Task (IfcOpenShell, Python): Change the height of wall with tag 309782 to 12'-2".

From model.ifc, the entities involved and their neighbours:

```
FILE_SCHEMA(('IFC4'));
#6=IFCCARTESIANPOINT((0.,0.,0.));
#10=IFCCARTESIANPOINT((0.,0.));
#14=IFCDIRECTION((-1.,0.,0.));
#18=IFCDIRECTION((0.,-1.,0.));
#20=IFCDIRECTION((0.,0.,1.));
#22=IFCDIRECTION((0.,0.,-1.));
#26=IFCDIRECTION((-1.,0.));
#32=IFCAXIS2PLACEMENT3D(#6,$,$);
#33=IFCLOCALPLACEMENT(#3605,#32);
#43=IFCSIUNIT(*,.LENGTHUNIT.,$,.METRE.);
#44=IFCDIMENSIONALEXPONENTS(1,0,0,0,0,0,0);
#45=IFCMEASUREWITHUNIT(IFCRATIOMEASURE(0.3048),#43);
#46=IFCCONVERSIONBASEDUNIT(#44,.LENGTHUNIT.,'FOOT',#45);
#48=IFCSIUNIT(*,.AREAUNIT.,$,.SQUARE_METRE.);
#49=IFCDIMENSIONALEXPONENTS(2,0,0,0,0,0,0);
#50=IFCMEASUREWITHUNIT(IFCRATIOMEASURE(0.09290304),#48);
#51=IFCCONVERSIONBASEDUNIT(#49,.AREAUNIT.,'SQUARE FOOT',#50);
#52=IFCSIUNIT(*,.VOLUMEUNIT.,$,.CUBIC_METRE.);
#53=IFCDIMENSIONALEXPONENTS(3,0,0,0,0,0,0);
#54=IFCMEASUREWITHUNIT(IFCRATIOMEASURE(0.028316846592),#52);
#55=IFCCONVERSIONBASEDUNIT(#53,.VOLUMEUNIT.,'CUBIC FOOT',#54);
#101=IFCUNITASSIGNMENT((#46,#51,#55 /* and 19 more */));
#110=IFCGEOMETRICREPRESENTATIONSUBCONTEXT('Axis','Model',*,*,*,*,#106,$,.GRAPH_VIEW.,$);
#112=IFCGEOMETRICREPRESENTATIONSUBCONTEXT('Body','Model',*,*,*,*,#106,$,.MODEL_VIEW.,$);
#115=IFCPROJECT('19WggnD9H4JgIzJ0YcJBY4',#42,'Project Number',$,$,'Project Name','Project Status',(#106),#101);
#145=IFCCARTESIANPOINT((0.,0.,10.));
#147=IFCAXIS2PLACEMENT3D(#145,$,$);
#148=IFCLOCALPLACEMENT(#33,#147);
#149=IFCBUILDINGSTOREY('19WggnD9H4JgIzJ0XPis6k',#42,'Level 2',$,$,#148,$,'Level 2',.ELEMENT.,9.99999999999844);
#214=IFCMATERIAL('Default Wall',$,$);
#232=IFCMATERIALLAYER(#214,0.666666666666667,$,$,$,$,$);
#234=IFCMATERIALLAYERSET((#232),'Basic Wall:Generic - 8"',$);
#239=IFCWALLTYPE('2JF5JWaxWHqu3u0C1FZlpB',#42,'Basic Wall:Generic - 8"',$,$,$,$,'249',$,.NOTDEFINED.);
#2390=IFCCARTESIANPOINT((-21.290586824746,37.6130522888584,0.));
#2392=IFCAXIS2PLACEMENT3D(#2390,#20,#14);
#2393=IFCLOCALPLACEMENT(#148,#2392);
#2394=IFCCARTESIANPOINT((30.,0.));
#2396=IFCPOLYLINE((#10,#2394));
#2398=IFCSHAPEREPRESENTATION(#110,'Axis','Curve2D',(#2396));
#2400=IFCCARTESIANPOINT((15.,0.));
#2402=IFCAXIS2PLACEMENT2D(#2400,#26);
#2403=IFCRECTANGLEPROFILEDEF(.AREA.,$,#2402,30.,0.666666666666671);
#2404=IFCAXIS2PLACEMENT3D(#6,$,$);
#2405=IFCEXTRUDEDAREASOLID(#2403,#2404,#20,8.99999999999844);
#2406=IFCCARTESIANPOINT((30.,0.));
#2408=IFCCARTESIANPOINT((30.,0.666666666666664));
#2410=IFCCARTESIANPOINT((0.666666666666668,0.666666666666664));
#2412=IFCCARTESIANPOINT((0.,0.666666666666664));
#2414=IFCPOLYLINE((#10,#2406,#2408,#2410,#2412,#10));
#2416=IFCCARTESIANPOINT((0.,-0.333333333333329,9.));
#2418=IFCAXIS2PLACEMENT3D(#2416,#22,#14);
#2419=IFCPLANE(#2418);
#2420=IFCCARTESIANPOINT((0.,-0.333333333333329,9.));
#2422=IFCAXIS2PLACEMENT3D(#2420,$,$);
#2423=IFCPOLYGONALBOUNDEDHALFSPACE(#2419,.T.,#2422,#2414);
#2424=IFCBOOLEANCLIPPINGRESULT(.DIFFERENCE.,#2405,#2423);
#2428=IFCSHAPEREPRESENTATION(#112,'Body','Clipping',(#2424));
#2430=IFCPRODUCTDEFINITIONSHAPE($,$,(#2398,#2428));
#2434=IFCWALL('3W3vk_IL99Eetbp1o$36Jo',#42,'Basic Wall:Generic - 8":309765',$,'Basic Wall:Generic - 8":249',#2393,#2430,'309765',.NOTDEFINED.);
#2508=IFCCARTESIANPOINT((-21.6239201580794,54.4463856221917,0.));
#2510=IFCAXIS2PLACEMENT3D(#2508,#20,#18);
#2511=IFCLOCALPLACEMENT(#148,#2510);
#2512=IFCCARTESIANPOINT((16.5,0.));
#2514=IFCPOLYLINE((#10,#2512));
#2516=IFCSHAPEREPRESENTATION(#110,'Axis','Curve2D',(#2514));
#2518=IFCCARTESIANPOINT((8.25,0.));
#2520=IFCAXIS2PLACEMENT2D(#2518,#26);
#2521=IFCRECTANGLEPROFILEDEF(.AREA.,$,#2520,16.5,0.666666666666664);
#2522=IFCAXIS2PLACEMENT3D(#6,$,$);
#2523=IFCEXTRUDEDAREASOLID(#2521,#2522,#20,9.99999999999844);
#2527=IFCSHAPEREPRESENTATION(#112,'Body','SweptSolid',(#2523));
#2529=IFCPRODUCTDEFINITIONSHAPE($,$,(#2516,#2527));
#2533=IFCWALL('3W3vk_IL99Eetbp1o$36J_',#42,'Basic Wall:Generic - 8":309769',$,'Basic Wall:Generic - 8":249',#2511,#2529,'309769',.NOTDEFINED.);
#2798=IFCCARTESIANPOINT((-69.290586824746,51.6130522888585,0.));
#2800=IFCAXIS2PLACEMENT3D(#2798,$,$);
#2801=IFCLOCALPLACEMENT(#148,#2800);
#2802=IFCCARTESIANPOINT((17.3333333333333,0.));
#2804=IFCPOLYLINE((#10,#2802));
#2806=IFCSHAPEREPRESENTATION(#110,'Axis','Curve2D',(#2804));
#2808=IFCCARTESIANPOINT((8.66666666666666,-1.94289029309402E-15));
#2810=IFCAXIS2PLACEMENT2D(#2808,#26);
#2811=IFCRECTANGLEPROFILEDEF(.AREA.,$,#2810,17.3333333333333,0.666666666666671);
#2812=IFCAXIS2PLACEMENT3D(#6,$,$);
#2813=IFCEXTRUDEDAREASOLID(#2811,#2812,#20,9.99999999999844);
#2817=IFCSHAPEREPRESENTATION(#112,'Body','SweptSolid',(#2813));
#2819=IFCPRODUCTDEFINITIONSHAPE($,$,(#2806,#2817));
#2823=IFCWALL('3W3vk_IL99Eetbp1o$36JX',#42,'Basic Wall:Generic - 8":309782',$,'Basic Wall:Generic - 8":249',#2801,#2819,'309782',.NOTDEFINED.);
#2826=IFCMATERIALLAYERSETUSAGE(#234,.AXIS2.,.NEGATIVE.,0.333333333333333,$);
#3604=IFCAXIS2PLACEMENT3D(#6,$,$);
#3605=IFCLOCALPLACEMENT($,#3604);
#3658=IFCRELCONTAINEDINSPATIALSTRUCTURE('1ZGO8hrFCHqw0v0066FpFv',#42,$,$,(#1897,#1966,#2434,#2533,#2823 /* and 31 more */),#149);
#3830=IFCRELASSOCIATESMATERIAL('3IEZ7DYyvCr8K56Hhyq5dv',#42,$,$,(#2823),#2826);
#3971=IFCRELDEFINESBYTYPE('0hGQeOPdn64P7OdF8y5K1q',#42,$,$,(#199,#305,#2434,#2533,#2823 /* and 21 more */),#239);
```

```python
import ifcopenshell
import ifcopenshell.geom
import ifcopenshell.util.representation
import ifcopenshell.util.shape
import ifcopenshell.util.unit

model = ifcopenshell.open("model.ifc")
unit_scale = ifcopenshell.util.unit.calculate_unit_scale(model)
settings = ifcopenshell.geom.settings()


def volume(element):
    """Net volume in cubic metres, openings subtracted."""
    shape = ifcopenshell.geom.create_shape(settings, element)
    return ifcopenshell.util.shape.get_volume(shape.geometry)


wall = model.by_guid("3W3vk_IL99Eetbp1o$36JX")
before = volume(wall)

body = ifcopenshell.util.representation.get_representation(wall, "Model", "Body")
solid = body.Items[0]
old_height = solid.Depth
solid.Depth = 146 * 0.0254 / unit_scale
after = volume(wall)

print(f"height {old_height:g} -> {solid.Depth:g}, volume {before:.3f} -> {after:.3f} m3")

model.write("model_rev.ifc")
```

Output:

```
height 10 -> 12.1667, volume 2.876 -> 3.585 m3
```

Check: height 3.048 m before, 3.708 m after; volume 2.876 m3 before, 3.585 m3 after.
